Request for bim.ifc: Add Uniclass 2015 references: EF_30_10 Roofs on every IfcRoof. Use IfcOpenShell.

First a look at what the model holds.

```python
import ifcopenshell

model = ifcopenshell.open("bim.ifc")
print(model.schema)
print("classifications:", [c.Name for c in model.by_type("IfcClassification")])
for ifc_class in ("IfcDoor", "IfcRoof", "IfcStair", "IfcWall", "IfcWindow"):
    print(ifc_class, len(model.by_type(ifc_class)))
```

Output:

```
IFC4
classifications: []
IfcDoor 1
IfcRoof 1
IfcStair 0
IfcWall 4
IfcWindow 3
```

```python
import ifcopenshell
import ifcopenshell.api.classification

model = ifcopenshell.open("bim.ifc")

system = ifcopenshell.api.classification.add_classification(model, classification="Uniclass 2015")

codes = {
    "IfcRoof": ("EF_30_10", "Roofs"),
}
for ifc_class, (code, name) in codes.items():
    products = model.by_type(ifc_class)
    ifcopenshell.api.classification.add_reference(
        model, products=products, classification=system, identification=code, name=name
    )
    print(code, len(products))

model.write("bim_updated.ifc")
```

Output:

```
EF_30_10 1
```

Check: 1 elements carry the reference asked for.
